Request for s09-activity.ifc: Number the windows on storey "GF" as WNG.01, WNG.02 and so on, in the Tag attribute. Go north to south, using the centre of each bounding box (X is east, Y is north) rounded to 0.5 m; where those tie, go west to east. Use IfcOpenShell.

First a look at what the model holds.

```python
import ifcopenshell
import ifcopenshell.util.element
import ifcopenshell.util.placement

model = ifcopenshell.open("s09-activity.ifc")
print(model.schema)
storey = next(s for s in model.by_type("IfcBuildingStorey") if s.Name == "GF")
windows = [e for e in ifcopenshell.util.element.get_decomposition(storey) if e.is_a("IfcWindow")]
for e in sorted(windows, key=lambda e: e.id()):
    origin = ifcopenshell.util.placement.get_local_placement(e.ObjectPlacement)[:3, 3]
    print(e.id(), e.Tag, e.Name, origin.round(2) + 0.0, sep=" | ")
```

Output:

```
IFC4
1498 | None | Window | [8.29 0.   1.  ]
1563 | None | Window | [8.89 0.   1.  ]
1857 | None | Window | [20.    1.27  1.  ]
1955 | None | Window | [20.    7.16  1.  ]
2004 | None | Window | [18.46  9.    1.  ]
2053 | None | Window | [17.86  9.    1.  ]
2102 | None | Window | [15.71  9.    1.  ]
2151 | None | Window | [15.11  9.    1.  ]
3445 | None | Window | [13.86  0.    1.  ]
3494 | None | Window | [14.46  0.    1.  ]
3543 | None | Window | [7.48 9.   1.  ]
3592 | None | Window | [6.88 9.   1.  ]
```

```python
import ifcopenshell
import ifcopenshell.geom
import ifcopenshell.util.element
import ifcopenshell.util.shape

model = ifcopenshell.open("s09-activity.ifc")
settings = ifcopenshell.geom.settings()
settings.set("use-world-coords", True)


def centre(element):
    shape = ifcopenshell.geom.create_shape(settings, element)
    return ifcopenshell.util.shape.get_bbox_centroid(shape.geometry)


storey = next(s for s in model.by_type("IfcBuildingStorey") if s.Name == "GF")
windows = [e for e in ifcopenshell.util.element.get_decomposition(storey) if e.is_a("IfcWindow")]

# Insertion points can sit at a corner or the storey origin, so sort by the geometry (in metres).
centres = {e: centre(e) for e in windows}
windows.sort(key=lambda e: (-round(centres[e][1] / 0.5), centres[e][0]))

for i, e in enumerate(windows, start=1):
    number = f"WNG.{i:02d}"
    e.Tag = number
    print(e.id(), number)

model.write("s09-activity_v2.ifc")
```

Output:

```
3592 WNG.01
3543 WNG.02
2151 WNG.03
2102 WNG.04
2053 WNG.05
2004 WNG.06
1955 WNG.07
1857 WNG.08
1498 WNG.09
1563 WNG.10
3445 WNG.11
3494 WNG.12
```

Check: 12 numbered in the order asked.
